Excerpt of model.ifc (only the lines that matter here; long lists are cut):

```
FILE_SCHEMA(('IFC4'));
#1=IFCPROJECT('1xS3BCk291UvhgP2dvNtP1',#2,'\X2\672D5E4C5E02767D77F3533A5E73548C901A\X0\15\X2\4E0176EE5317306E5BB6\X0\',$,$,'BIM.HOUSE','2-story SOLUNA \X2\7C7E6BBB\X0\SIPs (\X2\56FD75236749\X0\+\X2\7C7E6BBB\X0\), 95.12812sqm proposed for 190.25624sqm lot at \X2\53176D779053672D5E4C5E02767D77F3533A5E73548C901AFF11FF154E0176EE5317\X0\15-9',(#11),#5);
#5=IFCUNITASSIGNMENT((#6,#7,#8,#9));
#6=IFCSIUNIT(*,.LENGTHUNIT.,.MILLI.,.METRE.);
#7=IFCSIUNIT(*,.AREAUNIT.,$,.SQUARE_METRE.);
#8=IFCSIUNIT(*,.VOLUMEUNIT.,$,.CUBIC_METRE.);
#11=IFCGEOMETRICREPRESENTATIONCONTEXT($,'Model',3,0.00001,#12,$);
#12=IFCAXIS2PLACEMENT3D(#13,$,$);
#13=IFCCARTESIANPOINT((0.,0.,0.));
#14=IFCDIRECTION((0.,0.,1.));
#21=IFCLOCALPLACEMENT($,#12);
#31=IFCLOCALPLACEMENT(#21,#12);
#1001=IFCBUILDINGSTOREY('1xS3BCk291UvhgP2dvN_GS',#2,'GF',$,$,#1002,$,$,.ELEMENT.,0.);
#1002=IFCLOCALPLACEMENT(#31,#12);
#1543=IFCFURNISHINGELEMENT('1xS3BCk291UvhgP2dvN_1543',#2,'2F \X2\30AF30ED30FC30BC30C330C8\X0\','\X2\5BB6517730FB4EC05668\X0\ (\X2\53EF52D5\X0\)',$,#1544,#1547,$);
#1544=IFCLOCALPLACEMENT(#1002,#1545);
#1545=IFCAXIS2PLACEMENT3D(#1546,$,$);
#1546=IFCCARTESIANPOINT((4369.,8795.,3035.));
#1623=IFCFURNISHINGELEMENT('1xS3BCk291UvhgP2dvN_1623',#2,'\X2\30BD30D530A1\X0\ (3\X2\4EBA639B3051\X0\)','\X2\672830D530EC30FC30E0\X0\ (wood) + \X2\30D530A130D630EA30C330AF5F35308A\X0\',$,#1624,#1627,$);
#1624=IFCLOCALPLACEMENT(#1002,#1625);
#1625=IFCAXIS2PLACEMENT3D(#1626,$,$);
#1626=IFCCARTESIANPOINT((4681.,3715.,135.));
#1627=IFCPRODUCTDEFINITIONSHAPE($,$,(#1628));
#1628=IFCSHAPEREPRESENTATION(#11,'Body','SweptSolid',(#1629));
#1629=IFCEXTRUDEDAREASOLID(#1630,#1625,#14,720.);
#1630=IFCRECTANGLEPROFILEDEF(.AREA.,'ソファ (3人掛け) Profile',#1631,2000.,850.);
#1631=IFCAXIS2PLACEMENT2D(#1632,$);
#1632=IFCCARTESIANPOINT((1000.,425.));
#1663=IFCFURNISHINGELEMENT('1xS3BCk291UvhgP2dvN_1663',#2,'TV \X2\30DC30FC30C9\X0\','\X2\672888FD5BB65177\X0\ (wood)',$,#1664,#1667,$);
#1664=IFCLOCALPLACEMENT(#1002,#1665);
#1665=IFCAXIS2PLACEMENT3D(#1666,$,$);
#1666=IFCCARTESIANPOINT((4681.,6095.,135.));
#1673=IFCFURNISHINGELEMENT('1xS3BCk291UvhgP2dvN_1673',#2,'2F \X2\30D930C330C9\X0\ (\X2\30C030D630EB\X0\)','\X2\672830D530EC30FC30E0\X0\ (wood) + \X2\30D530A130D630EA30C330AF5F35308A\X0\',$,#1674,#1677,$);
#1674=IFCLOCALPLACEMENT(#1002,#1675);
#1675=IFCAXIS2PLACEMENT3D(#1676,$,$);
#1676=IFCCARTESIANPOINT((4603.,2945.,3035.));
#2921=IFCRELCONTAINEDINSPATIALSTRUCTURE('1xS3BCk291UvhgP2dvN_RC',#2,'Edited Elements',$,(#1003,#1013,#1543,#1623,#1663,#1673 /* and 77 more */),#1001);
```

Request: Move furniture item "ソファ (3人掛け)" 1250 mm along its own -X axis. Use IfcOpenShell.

```python
import ifcopenshell
import ifcopenshell.api.geometry
import ifcopenshell.util.placement
import ifcopenshell.util.unit

model = ifcopenshell.open("model.ifc")
unit_scale = ifcopenshell.util.unit.calculate_unit_scale(model)

item = model.by_guid("1xS3BCk291UvhgP2dvN_1623")
matrix = ifcopenshell.util.placement.get_local_placement(item.ObjectPlacement)
matrix[:3, 3] -= matrix[:3, 0] * 1.25 / unit_scale
ifcopenshell.api.geometry.edit_object_placement(model, product=item, matrix=matrix, is_si=False)

print(ifcopenshell.util.placement.get_local_placement(item.ObjectPlacement).round(3) + 0.0)

model.write("model_rev.ifc")
```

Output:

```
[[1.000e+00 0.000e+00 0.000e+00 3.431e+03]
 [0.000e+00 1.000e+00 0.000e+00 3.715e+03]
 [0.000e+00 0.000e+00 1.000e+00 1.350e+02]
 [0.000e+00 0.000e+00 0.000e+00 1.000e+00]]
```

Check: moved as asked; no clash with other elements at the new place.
